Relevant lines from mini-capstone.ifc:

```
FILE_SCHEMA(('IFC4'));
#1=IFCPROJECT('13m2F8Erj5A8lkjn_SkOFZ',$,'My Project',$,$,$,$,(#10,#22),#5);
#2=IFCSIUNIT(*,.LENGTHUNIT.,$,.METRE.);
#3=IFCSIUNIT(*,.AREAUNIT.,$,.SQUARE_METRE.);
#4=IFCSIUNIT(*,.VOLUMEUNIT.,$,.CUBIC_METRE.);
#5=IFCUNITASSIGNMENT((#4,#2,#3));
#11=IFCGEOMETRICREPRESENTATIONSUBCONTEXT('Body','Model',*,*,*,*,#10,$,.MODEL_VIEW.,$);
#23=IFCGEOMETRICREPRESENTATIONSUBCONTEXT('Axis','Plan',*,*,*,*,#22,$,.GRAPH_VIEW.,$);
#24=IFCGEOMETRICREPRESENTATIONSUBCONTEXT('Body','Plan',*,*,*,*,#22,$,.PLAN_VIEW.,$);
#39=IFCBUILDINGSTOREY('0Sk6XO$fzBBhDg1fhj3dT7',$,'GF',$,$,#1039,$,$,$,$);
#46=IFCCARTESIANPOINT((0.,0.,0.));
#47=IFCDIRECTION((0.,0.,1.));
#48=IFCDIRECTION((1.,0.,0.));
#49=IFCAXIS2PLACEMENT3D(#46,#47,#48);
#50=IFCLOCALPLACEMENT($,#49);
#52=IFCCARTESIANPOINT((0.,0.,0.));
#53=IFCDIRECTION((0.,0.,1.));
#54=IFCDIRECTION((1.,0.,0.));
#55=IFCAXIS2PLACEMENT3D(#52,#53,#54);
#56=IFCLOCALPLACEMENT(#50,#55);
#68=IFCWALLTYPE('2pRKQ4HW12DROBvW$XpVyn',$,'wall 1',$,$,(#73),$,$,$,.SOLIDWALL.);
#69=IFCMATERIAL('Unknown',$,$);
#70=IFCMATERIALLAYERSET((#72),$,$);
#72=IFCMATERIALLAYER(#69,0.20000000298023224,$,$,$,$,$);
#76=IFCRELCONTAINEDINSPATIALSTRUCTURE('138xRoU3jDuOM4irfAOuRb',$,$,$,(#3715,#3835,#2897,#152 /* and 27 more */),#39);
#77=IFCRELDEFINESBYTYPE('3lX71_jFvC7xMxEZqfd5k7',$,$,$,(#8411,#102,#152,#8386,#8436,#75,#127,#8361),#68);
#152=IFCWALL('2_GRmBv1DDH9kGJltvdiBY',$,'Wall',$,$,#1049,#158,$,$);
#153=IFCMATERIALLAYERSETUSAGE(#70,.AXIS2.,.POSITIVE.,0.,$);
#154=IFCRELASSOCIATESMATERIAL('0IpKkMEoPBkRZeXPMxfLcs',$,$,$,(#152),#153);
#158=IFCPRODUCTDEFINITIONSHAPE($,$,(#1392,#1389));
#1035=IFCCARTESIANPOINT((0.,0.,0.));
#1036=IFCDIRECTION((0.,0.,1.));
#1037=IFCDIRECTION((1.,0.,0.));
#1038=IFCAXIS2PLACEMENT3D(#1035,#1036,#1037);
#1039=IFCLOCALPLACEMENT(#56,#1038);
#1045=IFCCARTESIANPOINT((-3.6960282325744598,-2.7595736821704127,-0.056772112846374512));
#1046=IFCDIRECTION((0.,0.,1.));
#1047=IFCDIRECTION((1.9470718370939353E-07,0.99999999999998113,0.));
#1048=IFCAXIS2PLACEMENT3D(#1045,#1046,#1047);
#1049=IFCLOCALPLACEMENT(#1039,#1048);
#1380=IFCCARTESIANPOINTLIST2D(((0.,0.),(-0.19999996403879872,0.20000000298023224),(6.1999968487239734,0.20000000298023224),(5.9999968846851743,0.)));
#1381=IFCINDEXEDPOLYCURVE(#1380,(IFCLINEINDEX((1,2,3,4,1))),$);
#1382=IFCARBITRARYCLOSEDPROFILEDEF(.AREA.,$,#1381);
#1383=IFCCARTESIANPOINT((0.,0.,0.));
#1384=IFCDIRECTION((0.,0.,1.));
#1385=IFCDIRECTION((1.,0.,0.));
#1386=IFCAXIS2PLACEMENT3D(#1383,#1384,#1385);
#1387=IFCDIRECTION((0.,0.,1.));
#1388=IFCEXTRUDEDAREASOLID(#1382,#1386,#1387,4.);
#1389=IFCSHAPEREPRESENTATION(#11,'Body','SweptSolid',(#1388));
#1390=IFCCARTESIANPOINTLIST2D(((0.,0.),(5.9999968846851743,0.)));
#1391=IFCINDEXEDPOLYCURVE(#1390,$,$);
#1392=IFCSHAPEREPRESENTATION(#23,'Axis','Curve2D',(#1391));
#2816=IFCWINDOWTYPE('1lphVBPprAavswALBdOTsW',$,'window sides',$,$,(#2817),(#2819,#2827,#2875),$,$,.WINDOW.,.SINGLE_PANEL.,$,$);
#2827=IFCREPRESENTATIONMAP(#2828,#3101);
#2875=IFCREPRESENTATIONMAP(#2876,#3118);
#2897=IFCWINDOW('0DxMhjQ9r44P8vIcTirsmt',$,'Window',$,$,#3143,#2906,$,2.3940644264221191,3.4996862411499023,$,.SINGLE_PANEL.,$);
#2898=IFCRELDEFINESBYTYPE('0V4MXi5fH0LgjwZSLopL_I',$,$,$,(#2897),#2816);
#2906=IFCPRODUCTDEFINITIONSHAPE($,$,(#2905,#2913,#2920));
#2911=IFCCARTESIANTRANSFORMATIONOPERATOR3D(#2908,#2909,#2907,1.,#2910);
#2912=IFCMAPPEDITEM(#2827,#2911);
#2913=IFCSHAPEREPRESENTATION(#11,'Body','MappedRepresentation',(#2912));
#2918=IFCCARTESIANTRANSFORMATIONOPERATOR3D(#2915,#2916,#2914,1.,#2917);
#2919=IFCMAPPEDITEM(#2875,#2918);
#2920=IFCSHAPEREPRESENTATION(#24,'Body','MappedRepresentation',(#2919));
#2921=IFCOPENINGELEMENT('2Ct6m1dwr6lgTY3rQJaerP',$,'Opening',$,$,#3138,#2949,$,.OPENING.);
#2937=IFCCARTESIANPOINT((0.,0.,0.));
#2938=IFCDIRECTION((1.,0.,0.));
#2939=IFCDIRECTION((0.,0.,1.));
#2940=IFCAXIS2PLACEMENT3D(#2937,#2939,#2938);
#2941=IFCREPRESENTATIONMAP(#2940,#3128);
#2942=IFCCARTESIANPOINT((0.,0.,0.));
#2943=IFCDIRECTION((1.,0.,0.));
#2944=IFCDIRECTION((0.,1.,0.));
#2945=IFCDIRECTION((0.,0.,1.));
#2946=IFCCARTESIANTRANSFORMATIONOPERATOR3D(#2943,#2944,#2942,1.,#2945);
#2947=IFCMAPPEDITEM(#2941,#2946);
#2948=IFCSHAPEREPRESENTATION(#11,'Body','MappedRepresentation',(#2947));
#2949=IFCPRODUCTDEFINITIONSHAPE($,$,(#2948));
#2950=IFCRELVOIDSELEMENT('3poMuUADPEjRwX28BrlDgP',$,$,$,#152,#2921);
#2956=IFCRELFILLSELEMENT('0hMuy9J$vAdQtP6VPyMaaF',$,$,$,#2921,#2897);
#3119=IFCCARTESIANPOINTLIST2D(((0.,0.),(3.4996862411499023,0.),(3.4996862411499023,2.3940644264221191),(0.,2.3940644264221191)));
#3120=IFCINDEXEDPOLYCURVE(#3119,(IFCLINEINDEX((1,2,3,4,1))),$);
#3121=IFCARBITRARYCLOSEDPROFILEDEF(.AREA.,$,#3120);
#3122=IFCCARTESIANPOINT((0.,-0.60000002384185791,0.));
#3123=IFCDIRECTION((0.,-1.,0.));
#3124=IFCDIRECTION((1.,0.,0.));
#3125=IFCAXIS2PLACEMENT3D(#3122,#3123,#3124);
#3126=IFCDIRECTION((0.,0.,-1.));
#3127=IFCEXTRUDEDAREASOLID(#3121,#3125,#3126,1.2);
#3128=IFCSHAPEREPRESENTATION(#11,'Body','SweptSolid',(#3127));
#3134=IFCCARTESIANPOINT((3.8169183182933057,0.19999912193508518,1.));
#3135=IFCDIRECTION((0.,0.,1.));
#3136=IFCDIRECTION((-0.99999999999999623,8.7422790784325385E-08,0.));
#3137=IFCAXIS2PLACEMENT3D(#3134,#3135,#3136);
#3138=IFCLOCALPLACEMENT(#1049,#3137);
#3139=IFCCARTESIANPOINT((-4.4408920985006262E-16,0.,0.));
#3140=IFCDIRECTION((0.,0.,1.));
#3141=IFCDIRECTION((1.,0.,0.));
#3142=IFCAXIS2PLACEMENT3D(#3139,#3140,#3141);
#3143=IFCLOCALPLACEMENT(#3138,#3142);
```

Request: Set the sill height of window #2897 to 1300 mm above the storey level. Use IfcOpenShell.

```python
import numpy as np
import ifcopenshell
import ifcopenshell.api.geometry
import ifcopenshell.geom
import ifcopenshell.util.element
import ifcopenshell.util.placement
import ifcopenshell.util.shape
import ifcopenshell.util.unit

model = ifcopenshell.open("mini-capstone.ifc")
unit_scale = ifcopenshell.util.unit.calculate_unit_scale(model)

window = model.by_guid("0DxMhjQ9r44P8vIcTirsmt")
opening = window.FillsVoids[0].RelatingOpeningElement
storey = ifcopenshell.util.element.get_container(window, ifc_class="IfcBuildingStorey")
level = ifcopenshell.util.placement.get_local_placement(storey.ObjectPlacement)[2, 3]

# The opening's origin need not be at the sill, so measure its lowest point.
shape = ifcopenshell.geom.create_shape(ifcopenshell.geom.settings(), opening)
bottom = ifcopenshell.util.shape.get_shape_bottom_elevation(shape, shape.geometry) / unit_scale
dz = level + 1.3 / unit_scale - bottom

shift = np.array([0.0, 0.0, dz])
# The window is placed relative to its opening, so it follows when the opening moves.
matrix = ifcopenshell.util.placement.get_local_placement(opening.ObjectPlacement)
matrix[:3, 3] += shift
ifcopenshell.api.geometry.edit_object_placement(
    model, product=opening, matrix=matrix, is_si=False, should_transform_children=True
)

print(f"moved by {dz * unit_scale:+.3f} m")

model.write("mini-capstone_rev.ifc")
```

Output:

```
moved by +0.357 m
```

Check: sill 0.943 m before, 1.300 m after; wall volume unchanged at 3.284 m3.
